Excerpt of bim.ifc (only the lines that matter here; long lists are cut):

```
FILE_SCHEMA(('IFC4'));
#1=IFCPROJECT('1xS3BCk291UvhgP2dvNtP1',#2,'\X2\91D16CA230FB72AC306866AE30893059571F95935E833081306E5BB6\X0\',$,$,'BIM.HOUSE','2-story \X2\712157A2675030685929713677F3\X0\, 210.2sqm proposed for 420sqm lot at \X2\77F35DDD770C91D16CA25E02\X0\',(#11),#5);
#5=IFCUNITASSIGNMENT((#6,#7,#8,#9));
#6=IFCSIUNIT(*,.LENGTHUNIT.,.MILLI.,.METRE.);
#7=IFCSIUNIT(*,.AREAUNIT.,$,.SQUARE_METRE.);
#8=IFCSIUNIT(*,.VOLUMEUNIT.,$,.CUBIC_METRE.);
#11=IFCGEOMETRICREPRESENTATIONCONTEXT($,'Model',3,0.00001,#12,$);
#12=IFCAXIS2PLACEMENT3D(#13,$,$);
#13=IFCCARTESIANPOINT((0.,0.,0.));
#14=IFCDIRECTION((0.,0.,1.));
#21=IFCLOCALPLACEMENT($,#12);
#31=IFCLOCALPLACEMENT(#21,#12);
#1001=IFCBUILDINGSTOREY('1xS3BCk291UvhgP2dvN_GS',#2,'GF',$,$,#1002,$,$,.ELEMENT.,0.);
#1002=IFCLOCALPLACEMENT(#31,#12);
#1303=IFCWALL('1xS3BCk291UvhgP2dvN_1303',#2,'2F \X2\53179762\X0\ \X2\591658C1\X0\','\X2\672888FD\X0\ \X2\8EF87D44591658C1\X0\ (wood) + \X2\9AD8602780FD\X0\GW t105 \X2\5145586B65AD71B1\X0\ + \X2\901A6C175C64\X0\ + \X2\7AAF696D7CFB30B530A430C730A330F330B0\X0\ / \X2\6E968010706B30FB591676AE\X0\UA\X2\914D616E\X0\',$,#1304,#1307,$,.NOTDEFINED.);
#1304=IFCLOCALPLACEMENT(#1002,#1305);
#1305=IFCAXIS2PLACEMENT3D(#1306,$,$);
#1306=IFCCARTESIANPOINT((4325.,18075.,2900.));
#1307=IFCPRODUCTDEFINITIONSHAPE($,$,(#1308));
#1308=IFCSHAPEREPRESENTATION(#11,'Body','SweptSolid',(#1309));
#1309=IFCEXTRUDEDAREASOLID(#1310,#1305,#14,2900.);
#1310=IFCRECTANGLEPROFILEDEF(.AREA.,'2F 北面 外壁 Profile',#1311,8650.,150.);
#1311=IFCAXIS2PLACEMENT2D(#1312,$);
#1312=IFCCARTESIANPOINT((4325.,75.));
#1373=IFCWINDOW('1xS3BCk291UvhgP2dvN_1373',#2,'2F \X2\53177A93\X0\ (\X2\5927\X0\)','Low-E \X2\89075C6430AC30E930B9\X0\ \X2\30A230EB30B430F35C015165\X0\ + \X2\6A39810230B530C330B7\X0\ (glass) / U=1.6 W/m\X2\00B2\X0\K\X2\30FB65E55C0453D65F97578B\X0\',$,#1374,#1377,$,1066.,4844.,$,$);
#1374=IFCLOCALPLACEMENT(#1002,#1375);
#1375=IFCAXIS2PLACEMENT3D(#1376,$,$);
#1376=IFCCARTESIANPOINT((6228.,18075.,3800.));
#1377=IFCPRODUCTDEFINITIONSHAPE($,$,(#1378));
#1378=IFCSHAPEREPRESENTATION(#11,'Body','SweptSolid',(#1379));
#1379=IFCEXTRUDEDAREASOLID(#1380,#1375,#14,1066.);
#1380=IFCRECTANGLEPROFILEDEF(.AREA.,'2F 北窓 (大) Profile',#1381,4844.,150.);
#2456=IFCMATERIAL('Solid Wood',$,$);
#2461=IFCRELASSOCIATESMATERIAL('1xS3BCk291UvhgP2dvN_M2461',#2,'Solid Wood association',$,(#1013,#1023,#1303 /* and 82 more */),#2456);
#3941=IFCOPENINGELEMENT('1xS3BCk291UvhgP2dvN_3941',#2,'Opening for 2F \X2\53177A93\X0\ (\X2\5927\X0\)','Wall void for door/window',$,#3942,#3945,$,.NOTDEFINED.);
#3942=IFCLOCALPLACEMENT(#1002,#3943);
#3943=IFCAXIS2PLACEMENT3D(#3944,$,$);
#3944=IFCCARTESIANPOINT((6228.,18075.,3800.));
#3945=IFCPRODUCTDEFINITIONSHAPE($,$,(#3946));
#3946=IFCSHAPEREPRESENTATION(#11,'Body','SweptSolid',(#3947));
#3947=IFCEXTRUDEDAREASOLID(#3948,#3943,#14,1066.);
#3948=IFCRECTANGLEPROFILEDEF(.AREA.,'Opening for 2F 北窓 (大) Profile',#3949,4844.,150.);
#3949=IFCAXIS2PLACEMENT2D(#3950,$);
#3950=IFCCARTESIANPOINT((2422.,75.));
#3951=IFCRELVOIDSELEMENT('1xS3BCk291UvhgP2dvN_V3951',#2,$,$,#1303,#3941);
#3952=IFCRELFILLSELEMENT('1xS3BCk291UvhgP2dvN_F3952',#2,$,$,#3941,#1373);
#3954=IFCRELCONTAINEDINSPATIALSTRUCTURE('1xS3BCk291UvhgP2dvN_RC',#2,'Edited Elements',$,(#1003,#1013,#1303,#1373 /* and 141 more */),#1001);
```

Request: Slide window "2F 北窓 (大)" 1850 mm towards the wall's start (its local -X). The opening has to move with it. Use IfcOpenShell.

```python
import ifcopenshell
import ifcopenshell.api.geometry
import ifcopenshell.util.placement

model = ifcopenshell.open("bim.ifc")

window = model.by_guid("1xS3BCk291UvhgP2dvN_1373")
opening = window.FillsVoids[0].RelatingOpeningElement
wall = opening.VoidsElements[0].RelatingBuildingElement

wall_matrix = ifcopenshell.util.placement.get_local_placement(wall.ObjectPlacement)
shift = wall_matrix[:3, 0] * -1850.0
before = ifcopenshell.util.placement.get_local_placement(window.ObjectPlacement)[:3, 3].copy()

# The window is not placed relative to its opening, so move both.
for product in (opening, window):
    matrix = ifcopenshell.util.placement.get_local_placement(product.ObjectPlacement)
    matrix[:3, 3] += shift
    ifcopenshell.api.geometry.edit_object_placement(model, product=product, matrix=matrix, is_si=False)

after = ifcopenshell.util.placement.get_local_placement(window.ObjectPlacement)[:3, 3]
print("window moved by", (after - before).round(3) + 0.0)

model.write("bim-out.ifc")
```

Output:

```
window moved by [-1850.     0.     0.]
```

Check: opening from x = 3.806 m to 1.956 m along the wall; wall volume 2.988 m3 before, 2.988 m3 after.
